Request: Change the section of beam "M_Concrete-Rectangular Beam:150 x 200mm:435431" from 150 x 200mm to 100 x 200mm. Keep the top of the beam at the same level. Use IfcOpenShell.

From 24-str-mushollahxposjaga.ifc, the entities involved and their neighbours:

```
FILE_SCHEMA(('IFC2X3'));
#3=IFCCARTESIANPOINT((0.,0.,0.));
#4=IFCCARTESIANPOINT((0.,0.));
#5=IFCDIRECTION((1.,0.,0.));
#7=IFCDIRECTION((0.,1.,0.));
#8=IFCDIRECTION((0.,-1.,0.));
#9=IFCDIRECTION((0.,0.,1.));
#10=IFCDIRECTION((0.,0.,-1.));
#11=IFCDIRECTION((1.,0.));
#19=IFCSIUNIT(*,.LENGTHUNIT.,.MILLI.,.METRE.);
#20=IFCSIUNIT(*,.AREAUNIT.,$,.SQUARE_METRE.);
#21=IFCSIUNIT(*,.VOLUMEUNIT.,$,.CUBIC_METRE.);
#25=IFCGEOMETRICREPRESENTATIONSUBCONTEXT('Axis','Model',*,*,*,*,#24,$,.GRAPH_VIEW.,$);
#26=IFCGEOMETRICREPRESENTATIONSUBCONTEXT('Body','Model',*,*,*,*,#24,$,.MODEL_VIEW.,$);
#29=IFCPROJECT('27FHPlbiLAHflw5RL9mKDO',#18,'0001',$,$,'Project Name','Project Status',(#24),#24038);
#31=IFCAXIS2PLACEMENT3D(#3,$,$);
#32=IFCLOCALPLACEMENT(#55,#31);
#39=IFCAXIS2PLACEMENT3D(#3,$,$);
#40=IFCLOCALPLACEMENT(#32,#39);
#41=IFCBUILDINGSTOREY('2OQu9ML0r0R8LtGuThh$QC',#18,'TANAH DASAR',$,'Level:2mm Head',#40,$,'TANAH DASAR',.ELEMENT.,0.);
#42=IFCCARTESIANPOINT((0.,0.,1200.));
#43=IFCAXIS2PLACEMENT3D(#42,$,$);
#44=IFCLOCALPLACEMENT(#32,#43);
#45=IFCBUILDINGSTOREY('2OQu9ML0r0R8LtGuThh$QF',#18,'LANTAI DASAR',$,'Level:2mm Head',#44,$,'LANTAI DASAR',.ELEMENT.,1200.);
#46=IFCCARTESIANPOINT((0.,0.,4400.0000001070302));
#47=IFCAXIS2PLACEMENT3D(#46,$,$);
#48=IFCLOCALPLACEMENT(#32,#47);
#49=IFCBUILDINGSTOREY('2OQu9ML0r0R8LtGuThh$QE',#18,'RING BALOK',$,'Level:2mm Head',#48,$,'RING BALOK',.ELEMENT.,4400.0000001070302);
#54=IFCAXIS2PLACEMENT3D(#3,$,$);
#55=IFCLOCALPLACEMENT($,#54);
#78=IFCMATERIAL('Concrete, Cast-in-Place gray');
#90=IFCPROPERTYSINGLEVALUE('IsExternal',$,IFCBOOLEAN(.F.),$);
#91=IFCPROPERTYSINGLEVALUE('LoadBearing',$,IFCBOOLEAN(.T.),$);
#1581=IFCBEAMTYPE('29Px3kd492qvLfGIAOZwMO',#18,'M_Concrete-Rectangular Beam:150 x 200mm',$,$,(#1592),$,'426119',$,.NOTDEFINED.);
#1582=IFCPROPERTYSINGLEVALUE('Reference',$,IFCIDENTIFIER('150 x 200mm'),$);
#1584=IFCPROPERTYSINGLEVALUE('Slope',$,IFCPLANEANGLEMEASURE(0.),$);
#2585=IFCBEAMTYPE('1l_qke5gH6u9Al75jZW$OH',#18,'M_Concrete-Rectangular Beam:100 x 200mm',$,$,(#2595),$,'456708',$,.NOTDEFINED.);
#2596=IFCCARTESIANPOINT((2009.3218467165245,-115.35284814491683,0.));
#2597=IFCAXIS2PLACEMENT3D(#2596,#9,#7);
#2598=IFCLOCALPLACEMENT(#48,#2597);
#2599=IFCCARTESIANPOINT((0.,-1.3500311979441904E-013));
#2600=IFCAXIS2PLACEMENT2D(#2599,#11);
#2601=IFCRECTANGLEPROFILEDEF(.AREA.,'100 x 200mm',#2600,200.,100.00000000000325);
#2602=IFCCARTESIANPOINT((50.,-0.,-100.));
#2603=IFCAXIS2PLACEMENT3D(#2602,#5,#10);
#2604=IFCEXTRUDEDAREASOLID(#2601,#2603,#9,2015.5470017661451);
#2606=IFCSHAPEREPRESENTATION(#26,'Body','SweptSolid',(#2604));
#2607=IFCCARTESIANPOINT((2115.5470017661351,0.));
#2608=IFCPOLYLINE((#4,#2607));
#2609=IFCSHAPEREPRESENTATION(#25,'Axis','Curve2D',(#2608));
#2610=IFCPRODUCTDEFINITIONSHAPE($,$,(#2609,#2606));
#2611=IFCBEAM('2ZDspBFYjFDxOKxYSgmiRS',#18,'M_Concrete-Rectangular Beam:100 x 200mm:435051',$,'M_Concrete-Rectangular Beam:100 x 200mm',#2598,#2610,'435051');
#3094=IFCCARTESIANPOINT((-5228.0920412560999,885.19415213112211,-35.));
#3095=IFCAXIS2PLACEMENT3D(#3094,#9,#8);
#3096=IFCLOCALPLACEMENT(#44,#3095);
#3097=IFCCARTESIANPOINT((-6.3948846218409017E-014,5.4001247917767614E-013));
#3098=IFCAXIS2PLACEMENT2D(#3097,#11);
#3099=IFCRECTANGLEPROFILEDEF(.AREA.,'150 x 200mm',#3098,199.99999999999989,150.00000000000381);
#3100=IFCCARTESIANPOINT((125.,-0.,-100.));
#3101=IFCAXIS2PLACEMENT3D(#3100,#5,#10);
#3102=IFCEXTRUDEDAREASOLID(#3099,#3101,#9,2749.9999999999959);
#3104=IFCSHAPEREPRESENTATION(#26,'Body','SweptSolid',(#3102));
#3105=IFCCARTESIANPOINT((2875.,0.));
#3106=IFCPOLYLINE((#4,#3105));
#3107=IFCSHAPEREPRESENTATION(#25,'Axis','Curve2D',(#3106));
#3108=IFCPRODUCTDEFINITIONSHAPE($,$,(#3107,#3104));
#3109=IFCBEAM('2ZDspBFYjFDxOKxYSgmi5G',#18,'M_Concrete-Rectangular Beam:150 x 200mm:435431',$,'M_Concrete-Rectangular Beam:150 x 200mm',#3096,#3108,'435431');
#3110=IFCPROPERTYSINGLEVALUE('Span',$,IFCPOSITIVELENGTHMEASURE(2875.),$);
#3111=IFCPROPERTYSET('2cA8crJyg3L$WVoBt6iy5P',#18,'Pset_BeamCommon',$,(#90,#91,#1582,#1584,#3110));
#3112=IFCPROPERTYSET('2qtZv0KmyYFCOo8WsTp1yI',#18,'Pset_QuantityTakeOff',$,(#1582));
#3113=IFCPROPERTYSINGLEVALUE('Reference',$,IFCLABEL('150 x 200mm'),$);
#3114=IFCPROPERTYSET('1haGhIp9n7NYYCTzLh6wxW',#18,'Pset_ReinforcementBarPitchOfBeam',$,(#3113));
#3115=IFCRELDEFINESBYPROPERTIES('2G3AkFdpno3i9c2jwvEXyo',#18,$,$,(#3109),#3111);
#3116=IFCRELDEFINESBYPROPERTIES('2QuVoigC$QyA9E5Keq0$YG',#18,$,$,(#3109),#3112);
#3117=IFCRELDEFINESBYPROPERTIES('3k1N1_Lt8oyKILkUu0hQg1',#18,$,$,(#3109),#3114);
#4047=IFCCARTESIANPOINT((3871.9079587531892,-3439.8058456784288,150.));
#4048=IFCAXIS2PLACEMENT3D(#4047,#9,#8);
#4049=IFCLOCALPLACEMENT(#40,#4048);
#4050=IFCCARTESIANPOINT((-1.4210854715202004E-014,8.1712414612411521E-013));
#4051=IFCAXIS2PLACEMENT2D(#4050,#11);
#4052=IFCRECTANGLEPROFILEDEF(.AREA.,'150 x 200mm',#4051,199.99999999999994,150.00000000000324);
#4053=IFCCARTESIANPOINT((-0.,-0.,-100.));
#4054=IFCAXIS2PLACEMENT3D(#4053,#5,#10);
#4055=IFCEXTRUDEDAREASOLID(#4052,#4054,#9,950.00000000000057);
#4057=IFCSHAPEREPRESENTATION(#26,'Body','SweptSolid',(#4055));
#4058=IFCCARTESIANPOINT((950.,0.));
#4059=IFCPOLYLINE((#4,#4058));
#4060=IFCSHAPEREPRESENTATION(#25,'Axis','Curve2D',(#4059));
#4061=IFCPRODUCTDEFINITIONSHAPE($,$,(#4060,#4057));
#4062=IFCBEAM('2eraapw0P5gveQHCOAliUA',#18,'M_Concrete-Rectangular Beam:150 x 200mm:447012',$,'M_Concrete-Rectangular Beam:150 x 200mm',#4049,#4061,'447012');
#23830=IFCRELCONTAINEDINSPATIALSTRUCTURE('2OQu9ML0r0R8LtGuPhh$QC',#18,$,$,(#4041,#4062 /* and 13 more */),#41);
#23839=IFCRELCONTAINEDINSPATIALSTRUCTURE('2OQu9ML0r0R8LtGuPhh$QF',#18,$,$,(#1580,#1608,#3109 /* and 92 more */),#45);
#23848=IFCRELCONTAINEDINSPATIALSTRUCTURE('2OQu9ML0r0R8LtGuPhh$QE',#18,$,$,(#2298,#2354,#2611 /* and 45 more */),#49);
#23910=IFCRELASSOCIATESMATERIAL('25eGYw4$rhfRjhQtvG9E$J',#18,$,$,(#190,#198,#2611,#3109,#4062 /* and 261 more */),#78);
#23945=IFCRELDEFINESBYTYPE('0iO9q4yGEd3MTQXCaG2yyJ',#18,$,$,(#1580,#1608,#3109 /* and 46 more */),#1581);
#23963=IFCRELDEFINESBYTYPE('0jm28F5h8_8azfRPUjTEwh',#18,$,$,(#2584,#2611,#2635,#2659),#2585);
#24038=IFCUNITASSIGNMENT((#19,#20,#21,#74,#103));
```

```python
import ifcopenshell
import ifcopenshell.api.pset
import ifcopenshell.api.type
import ifcopenshell.util.element
import ifcopenshell.util.representation

model = ifcopenshell.open("24-str-mushollahxposjaga.ifc")

member = model.by_guid("2ZDspBFYjFDxOKxYSgmi5G")
source = next(p for p in model.by_type("IfcRectangleProfileDef") if p.ProfileName == "100 x 200mm")

body = ifcopenshell.util.representation.get_representation(member, "Model", "Body")
solid = body.Items[0]
old_profile = solid.SweptArea

# Copy the section's sizes but keep this member's own profile position.
profile = ifcopenshell.util.element.copy(model, source)
# Profiles are centred, so shift by half the change in depth to hold the top.
shift = (old_profile.XDim - profile.XDim) / 2
x, y = old_profile.Position.Location.Coordinates
up = (-1.0, 0.0)  # upwards, in the solid's own plane
location = model.createIfcCartesianPoint((x + up[0] * shift, y + up[1] * shift))
profile.Position = model.createIfcAxis2Placement2D(location, old_profile.Position.RefDirection)
solid.SweptArea = profile
if not model.get_total_inverses(old_profile):
    ifcopenshell.util.element.remove_deep2(model, old_profile)

new_type = model.by_guid("1l_qke5gH6u9Al75jZW$OH")
ifcopenshell.api.type.assign_type(
    model, related_objects=[member], relating_type=new_type, should_map_representations=False
)
member.Name = member.Name.replace("150 x 200mm", "100 x 200mm")
member.ObjectType = "M_Concrete-Rectangular Beam:100 x 200mm"
pset = model.by_id(ifcopenshell.util.element.get_pset(member, "Pset_BeamCommon", should_inherit=False)["id"])
ifcopenshell.api.pset.edit_pset(model, pset=pset, properties={"Reference": "100 x 200mm"})
pset = model.by_id(ifcopenshell.util.element.get_pset(member, "Pset_QuantityTakeOff", should_inherit=False)["id"])
ifcopenshell.api.pset.edit_pset(model, pset=pset, properties={"Reference": "100 x 200mm"})
pset = model.by_id(ifcopenshell.util.element.get_pset(member, "Pset_ReinforcementBarPitchOfBeam", should_inherit=False)["id"])
ifcopenshell.api.pset.edit_pset(model, pset=pset, properties={"Reference": "100 x 200mm"})

print(solid.SweptArea)

model.write("24-str-mushollahxposjaga_rev.ifc")
```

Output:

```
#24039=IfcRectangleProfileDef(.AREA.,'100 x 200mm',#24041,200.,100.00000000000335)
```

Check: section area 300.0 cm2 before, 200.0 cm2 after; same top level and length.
